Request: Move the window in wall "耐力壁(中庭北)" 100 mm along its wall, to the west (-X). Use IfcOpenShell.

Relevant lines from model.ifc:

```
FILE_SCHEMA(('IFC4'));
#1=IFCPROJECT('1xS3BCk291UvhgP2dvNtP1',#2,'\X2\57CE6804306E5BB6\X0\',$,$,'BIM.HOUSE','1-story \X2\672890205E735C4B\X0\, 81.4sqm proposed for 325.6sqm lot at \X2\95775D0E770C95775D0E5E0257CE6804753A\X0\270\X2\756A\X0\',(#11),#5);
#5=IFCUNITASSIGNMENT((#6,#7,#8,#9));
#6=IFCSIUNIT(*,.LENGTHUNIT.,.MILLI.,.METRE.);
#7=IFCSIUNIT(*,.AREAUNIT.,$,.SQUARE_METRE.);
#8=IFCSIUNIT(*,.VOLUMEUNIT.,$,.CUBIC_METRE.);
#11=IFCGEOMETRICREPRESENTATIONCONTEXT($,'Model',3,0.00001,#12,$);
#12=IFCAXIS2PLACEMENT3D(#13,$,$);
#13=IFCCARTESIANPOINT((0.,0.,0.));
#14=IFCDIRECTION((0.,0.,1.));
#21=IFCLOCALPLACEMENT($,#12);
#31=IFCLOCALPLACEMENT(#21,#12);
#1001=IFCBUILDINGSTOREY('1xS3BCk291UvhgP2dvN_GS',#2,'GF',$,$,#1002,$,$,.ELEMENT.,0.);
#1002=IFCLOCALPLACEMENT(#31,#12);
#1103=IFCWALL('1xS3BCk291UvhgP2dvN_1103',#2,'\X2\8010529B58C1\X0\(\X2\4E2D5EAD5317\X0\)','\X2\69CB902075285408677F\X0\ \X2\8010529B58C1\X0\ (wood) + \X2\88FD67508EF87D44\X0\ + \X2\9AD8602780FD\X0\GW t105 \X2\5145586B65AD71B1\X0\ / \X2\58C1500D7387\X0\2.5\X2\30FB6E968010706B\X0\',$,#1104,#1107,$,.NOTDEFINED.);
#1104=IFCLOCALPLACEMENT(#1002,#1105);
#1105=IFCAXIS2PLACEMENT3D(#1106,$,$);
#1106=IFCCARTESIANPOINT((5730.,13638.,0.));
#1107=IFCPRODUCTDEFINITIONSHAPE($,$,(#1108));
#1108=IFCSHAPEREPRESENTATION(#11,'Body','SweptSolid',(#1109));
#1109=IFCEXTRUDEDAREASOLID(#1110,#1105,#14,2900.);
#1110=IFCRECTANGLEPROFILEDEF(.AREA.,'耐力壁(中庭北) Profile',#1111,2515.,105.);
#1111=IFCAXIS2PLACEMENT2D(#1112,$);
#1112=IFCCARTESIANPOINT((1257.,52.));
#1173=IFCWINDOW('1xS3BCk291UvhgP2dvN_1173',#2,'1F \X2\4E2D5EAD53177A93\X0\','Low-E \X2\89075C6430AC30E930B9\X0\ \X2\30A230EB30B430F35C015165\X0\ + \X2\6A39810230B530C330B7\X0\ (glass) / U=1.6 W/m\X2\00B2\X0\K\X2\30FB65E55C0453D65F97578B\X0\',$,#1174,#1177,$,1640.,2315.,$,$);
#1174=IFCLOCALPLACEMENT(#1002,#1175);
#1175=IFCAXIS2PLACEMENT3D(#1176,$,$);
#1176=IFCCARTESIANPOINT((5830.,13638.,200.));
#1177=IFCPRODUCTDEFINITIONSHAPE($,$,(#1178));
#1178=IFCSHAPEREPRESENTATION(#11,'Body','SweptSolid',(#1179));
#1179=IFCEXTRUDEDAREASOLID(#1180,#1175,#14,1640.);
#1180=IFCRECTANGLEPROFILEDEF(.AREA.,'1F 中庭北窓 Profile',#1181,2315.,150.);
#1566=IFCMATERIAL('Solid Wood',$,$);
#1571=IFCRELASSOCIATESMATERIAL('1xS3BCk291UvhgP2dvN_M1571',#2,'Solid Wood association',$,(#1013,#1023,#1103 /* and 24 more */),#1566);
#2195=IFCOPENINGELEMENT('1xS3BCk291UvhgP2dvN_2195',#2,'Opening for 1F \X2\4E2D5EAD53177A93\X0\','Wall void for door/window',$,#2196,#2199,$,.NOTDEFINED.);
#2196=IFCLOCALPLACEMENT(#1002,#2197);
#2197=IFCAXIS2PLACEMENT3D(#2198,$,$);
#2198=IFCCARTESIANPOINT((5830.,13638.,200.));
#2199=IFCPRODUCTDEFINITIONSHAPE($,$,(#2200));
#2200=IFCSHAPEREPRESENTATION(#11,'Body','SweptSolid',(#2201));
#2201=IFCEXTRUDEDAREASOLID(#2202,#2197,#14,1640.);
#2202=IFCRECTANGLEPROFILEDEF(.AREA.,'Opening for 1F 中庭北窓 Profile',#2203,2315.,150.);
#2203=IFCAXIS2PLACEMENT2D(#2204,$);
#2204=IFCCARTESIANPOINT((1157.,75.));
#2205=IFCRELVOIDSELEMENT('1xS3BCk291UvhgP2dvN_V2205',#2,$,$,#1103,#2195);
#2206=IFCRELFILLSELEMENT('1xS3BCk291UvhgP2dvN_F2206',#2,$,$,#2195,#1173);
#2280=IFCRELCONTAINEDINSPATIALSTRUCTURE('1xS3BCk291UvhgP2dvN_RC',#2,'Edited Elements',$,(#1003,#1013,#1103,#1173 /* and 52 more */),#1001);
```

```python
import ifcopenshell
import ifcopenshell.api.geometry
import ifcopenshell.util.placement

model = ifcopenshell.open("model.ifc")

window = model.by_guid("1xS3BCk291UvhgP2dvN_1173")
opening = window.FillsVoids[0].RelatingOpeningElement
wall = opening.VoidsElements[0].RelatingBuildingElement

wall_matrix = ifcopenshell.util.placement.get_local_placement(wall.ObjectPlacement)
shift = wall_matrix[:3, 0] * -100.0
before = ifcopenshell.util.placement.get_local_placement(window.ObjectPlacement)[:3, 3].copy()

# The window is not placed relative to its opening, so move both.
for product in (opening, window):
    matrix = ifcopenshell.util.placement.get_local_placement(product.ObjectPlacement)
    matrix[:3, 3] += shift
    ifcopenshell.api.geometry.edit_object_placement(model, product=product, matrix=matrix, is_si=False)

after = ifcopenshell.util.placement.get_local_placement(window.ObjectPlacement)[:3, 3]
print("window moved by", (after - before).round(3) + 0.0)

model.write("model_v2.ifc")
```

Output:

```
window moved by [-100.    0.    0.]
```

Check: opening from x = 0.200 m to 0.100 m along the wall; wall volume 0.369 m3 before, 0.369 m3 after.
